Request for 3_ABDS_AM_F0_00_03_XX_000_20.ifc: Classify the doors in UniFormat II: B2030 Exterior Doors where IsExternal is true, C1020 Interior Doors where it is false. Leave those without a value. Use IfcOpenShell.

First a look at what the model holds.

```python
import ifcopenshell
import ifcopenshell.util.element

model = ifcopenshell.open("3_ABDS_AM_F0_00_03_XX_000_20.ifc")
print(model.schema)
print("classifications:", [c.Name for c in model.by_type("IfcClassification")])
values = [ifcopenshell.util.element.get_pset(e, "Pset_DoorCommon", "IsExternal") for e in model.by_type("IfcDoor")]
for value in (True, False, None):
    print("IsExternal", value, values.count(value))
```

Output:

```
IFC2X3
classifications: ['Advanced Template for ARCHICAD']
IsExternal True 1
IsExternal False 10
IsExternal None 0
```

```python
import ifcopenshell
import ifcopenshell.api.classification
import ifcopenshell.util.element

model = ifcopenshell.open("3_ABDS_AM_F0_00_03_XX_000_20.ifc")

# IFC2X3 requires Source and Edition and has no link from the project to the system.
system = model.create_entity("IfcClassification", Source="ASTM", Edition="E1557", Name="UniFormat II")

doors = model.by_type("IfcDoor")
external = {e: ifcopenshell.util.element.get_pset(e, "Pset_DoorCommon", "IsExternal") for e in doors}
for flag, code, name in ((True, "B2030", "Exterior Doors"), (False, "C1020", "Interior Doors")):
    products = [e for e in doors if external[e] is flag]
    ifcopenshell.api.classification.add_reference(
        model, products=products, classification=system, identification=code, name=name
    )
    print(code, len(products))

model.write("3_ABDS_AM_F0_00_03_XX_000_20_rev.ifc")
```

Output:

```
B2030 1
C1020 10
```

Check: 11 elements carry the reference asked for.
